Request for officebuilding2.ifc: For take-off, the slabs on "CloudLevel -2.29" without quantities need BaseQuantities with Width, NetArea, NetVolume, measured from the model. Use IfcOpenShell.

First a look at what the model holds.

```python
import ifcopenshell
import ifcopenshell.util.element
import ifcopenshell.util.unit

model = ifcopenshell.open("officebuilding2.ifc")
print(model.schema)
for unit_type in ("LENGTHUNIT", "AREAUNIT", "VOLUMEUNIT"):
    print(unit_type, ifcopenshell.util.unit.calculate_unit_scale(model, unit_type))
storey = next(s for s in model.by_type("IfcBuildingStorey") if s.Name == "CloudLevel -2.29")
slabs = [e for e in ifcopenshell.util.element.get_decomposition(storey) if e.is_a("IfcSlab")]
for e in sorted(slabs, key=lambda e: e.id()):
    print(e.id(), e.is_a(), e.Name, list(ifcopenshell.util.element.get_psets(e, qtos_only=True)), sep=" | ")
```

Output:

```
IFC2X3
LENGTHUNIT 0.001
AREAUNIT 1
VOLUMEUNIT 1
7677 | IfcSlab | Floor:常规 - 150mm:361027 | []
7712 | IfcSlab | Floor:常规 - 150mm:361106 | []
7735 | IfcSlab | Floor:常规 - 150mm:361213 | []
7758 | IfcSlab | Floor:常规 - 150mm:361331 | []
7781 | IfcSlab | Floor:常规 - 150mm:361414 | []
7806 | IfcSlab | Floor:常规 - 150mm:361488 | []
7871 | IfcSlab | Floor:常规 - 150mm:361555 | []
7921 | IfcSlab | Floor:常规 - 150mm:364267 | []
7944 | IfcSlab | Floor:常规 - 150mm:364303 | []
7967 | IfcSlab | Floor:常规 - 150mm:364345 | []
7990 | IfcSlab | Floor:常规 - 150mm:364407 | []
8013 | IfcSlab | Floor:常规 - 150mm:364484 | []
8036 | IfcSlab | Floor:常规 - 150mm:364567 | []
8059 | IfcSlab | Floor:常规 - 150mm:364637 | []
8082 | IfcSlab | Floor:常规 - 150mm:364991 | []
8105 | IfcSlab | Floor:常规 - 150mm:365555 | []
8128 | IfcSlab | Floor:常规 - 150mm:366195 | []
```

```python
import ifcopenshell
import ifcopenshell.api.pset
import ifcopenshell.geom
import ifcopenshell.util.element
import ifcopenshell.util.shape
import ifcopenshell.util.unit

model = ifcopenshell.open("officebuilding2.ifc")
unit_scale = ifcopenshell.util.unit.calculate_unit_scale(model)
area_scale = ifcopenshell.util.unit.calculate_unit_scale(model, "AREAUNIT")
volume_scale = ifcopenshell.util.unit.calculate_unit_scale(model, "VOLUMEUNIT")
settings = ifcopenshell.geom.settings()

storey = next(s for s in model.by_type("IfcBuildingStorey") if s.Name == "CloudLevel -2.29")
slabs = [e for e in ifcopenshell.util.element.get_decomposition(storey) if e.is_a("IfcSlab")]

for e in sorted(slabs, key=lambda e: e.id()):
    if ifcopenshell.util.element.get_psets(e, qtos_only=True, should_inherit=False):
        continue
    # Geometry comes back in metres, in the element's own axes.
    shape = ifcopenshell.geom.create_shape(settings, e)
    values = {
        "Width": ifcopenshell.util.shape.get_z(shape.geometry) / unit_scale,
        "NetArea": ifcopenshell.util.shape.get_footprint_area(shape.geometry) / area_scale,
        "NetVolume": ifcopenshell.util.shape.get_volume(shape.geometry) / volume_scale,
    }
    qto = ifcopenshell.api.pset.add_qto(model, product=e, name="BaseQuantities")
    ifcopenshell.api.pset.edit_qto(model, qto=qto, properties=values)
    print(e.id(), {k: round(v, 3) for k, v in values.items()})

model.write("officebuilding2_v2.ifc")
```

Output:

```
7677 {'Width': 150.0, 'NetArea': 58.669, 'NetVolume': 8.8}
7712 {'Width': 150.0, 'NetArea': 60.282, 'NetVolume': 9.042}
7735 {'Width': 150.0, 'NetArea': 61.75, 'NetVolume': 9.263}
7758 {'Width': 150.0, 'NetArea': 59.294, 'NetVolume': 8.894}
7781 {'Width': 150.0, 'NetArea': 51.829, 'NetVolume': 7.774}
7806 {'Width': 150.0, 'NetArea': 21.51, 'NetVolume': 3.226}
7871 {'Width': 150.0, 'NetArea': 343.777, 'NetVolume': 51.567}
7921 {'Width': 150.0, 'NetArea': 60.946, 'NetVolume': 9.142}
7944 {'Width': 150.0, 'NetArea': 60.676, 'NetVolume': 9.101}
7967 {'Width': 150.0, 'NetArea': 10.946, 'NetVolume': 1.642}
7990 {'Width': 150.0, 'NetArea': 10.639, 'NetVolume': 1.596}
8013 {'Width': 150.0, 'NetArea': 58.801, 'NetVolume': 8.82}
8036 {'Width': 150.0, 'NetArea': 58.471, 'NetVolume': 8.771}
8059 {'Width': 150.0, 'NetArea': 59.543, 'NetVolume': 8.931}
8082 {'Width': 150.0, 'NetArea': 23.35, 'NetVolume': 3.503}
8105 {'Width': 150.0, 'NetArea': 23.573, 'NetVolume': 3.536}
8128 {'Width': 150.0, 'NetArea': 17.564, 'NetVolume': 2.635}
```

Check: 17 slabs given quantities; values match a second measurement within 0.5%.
